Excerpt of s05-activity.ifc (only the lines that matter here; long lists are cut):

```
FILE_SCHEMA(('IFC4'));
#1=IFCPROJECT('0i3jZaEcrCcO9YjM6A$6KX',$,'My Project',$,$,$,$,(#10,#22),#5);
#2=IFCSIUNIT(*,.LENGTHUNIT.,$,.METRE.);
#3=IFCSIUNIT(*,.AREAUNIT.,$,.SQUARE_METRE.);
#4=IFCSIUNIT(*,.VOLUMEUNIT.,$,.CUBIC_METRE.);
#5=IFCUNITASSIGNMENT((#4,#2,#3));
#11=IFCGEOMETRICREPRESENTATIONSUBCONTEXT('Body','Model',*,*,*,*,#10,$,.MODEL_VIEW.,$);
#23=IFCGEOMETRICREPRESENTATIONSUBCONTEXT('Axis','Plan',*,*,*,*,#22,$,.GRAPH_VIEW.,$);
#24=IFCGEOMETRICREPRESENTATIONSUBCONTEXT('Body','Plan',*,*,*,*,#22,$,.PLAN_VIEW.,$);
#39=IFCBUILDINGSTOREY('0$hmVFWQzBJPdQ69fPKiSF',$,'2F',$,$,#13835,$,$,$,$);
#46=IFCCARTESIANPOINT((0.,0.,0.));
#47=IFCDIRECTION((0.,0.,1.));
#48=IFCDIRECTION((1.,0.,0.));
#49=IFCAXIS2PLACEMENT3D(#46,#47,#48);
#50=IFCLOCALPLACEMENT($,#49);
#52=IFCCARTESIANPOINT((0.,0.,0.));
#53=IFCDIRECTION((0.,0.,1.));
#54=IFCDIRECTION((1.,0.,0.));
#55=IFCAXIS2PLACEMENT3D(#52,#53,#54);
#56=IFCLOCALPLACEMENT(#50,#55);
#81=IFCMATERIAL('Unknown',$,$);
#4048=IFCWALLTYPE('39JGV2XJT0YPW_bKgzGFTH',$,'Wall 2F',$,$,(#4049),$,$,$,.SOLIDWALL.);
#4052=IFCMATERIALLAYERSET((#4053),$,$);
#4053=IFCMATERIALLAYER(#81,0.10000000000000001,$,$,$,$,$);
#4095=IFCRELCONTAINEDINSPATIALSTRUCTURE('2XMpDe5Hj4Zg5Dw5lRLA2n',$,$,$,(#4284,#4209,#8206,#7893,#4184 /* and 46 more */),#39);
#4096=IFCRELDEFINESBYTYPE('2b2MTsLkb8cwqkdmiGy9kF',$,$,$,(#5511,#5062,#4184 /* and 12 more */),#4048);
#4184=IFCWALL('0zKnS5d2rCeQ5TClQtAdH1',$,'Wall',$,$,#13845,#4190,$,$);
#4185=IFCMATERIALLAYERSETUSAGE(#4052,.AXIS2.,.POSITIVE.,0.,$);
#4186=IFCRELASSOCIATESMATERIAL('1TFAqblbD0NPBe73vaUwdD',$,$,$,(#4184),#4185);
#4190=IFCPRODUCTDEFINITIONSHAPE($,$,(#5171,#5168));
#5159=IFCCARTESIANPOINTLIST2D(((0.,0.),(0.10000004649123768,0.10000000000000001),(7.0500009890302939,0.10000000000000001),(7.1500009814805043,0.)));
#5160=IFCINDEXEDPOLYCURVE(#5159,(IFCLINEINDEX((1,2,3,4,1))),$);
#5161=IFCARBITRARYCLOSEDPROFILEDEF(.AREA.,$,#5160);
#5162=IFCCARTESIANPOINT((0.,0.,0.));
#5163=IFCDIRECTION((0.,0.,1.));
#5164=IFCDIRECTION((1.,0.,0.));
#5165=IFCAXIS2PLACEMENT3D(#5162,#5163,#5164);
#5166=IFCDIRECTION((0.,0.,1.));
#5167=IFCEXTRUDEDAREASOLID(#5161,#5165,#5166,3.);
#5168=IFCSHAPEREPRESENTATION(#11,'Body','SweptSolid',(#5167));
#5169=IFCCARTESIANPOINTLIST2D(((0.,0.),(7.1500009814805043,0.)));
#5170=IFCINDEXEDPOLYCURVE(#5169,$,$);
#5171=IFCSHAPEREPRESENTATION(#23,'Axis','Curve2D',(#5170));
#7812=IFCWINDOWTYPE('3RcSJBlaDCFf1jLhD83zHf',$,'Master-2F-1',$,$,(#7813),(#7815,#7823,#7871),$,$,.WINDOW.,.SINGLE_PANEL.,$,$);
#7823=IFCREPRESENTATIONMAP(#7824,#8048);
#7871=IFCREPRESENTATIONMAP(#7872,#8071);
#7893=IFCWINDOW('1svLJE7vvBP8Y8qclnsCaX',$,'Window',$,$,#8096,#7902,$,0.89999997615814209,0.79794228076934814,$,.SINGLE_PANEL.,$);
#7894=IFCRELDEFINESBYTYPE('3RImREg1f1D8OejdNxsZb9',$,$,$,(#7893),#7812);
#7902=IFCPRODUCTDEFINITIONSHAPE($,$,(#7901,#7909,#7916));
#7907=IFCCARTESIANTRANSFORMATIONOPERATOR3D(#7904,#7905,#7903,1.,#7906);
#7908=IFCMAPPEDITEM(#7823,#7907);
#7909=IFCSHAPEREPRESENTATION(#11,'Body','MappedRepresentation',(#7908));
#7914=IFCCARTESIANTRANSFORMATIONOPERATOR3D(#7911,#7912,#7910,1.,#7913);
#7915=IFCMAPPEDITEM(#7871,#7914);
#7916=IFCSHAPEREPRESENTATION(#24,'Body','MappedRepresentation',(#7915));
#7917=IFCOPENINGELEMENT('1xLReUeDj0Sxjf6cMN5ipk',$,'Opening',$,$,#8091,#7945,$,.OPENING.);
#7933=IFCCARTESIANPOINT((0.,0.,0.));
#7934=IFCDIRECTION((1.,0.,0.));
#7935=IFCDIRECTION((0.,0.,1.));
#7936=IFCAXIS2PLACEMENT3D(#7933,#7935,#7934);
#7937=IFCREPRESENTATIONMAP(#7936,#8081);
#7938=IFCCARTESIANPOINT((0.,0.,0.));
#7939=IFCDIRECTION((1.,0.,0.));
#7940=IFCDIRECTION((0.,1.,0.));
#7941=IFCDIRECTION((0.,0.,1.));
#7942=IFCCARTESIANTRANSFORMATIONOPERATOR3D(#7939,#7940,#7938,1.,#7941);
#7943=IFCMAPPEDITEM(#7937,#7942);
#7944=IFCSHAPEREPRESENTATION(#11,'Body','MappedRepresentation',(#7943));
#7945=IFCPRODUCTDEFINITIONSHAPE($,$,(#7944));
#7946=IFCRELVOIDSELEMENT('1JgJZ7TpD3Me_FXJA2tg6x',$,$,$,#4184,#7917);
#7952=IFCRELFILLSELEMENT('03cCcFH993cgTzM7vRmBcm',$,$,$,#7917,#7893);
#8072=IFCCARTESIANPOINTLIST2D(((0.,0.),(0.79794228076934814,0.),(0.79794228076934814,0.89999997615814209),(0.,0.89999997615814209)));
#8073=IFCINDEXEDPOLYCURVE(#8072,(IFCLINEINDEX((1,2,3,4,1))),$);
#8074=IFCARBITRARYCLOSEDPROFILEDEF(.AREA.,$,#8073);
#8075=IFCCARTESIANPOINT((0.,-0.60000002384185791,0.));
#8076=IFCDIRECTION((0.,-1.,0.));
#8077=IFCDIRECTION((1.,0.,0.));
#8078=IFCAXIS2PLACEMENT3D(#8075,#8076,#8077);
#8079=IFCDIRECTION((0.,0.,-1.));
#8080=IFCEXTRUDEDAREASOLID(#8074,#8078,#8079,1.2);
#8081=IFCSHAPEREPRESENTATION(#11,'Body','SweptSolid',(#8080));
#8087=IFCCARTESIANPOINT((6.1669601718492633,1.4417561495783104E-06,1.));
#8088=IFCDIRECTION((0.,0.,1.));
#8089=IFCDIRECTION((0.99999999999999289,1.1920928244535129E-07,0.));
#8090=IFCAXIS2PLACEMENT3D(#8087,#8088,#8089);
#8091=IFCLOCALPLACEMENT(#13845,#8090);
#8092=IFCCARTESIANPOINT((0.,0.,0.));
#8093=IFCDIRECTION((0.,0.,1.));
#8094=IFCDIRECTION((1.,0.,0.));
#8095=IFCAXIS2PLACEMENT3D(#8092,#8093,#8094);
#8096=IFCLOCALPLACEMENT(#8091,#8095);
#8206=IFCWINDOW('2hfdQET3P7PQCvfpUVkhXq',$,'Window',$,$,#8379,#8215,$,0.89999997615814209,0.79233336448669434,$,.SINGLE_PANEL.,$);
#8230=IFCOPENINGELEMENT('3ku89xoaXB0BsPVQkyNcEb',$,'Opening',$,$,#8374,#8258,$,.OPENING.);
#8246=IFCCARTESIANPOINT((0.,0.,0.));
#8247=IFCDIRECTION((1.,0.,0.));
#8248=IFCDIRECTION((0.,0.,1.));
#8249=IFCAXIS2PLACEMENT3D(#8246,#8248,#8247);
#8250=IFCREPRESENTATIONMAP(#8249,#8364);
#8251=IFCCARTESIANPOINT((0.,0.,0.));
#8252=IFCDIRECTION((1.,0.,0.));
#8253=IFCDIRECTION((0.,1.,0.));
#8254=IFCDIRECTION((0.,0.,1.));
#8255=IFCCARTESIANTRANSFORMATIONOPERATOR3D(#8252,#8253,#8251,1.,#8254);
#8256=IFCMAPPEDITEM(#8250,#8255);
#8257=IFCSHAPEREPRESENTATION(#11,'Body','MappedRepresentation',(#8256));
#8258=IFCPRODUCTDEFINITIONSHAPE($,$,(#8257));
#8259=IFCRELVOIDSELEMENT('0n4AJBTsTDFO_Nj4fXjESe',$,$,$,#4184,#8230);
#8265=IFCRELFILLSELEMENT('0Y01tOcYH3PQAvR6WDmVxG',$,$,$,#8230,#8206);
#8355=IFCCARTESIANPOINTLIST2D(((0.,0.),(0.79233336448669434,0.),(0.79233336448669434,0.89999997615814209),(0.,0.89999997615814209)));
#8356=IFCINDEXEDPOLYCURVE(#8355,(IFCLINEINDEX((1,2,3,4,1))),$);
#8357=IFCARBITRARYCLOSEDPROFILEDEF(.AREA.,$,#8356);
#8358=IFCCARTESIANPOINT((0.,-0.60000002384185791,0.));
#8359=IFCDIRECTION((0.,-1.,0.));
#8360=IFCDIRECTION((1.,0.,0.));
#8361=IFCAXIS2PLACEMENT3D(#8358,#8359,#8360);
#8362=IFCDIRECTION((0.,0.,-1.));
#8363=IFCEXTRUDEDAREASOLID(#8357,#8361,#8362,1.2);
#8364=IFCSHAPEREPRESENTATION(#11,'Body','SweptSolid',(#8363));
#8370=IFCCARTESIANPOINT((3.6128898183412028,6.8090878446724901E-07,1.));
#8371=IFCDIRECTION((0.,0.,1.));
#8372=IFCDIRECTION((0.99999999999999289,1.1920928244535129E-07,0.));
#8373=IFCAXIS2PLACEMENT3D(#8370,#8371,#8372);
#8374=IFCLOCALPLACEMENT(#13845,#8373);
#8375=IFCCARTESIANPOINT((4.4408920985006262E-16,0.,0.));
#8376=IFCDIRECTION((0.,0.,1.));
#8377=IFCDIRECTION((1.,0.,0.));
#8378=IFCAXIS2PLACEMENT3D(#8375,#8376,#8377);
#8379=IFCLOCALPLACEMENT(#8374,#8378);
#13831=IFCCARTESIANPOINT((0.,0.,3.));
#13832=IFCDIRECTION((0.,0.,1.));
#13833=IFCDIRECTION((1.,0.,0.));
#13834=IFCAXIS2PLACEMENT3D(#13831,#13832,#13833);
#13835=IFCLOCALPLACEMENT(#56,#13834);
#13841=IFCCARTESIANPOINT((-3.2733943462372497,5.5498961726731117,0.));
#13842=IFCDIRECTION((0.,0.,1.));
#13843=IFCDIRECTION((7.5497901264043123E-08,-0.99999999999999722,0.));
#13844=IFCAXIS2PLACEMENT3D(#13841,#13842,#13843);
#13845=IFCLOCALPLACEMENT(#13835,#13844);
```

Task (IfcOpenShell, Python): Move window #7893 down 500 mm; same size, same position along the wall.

```python
import numpy as np
import ifcopenshell
import ifcopenshell.api.geometry
import ifcopenshell.util.placement
import ifcopenshell.util.unit

model = ifcopenshell.open("s05-activity.ifc")
unit_scale = ifcopenshell.util.unit.calculate_unit_scale(model)

window = model.by_guid("1svLJE7vvBP8Y8qclnsCaX")
opening = window.FillsVoids[0].RelatingOpeningElement
dz = -0.5 / unit_scale

shift = np.array([0.0, 0.0, dz])
# The window is placed relative to its opening, so it follows when the opening moves.
matrix = ifcopenshell.util.placement.get_local_placement(opening.ObjectPlacement)
matrix[:3, 3] += shift
ifcopenshell.api.geometry.edit_object_placement(
    model, product=opening, matrix=matrix, is_si=False, should_transform_children=True
)

print(f"moved by {dz * unit_scale:+.3f} m")

model.write("s05-activity_rev.ifc")
```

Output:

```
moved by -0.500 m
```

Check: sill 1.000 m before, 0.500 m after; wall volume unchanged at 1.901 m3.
